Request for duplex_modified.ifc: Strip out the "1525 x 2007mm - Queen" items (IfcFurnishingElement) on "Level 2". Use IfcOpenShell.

First a look at what the model holds.

```python
import ifcopenshell
import ifcopenshell.util.element

model = ifcopenshell.open("duplex_modified.ifc")
print(model.schema)
storey = next(s for s in model.by_type("IfcBuildingStorey") if s.Name == "Level 2")
furniture = [e for e in ifcopenshell.util.element.get_decomposition(storey) if e.is_a("IfcFurnishingElement")]
seen = {}
for e in furniture:
    element_type = ifcopenshell.util.element.get_type(e)
    name = element_type.Name if element_type not in (None, e) else None
    seen[name] = seen.get(name, 0) + 1
for name, count in sorted(seen.items(), key=str):
    print(count, "x", name)
```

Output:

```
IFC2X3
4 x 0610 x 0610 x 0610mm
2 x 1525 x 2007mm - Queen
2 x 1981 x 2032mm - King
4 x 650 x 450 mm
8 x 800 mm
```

```python
import ifcopenshell
import ifcopenshell.api.root
import ifcopenshell.util.element

model = ifcopenshell.open("duplex_modified.ifc")

storey = next(s for s in model.by_type("IfcBuildingStorey") if s.Name == "Level 2")
furniture = [e for e in ifcopenshell.util.element.get_decomposition(storey) if e.is_a("IfcFurnishingElement")]
targets = [e for e in furniture if (t := ifcopenshell.util.element.get_type(e)) not in (None, e) and t.Name == "1525 x 2007mm - Queen"]

for e in targets:
    ifcopenshell.api.root.remove_product(model, product=e)
print(len(targets), "removed")

model.write("duplex_modified_v2.ifc")
```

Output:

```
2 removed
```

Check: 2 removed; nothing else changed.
